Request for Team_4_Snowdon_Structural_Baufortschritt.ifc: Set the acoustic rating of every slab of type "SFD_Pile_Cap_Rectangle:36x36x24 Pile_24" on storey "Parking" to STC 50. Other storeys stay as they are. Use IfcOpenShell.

First a look at what the model holds.

```python
import ifcopenshell
import ifcopenshell.util.element

model = ifcopenshell.open("Team_4_Snowdon_Structural_Baufortschritt.ifc")
print(model.schema)
storey = next(s for s in model.by_type("IfcBuildingStorey") if s.Name == "Parking")
slabs = [e for e in ifcopenshell.util.element.get_decomposition(storey) if e.is_a("IfcSlab")]
seen = {}
for e in slabs:
    element_type = ifcopenshell.util.element.get_type(e)
    key = (element_type.Name if element_type != e and element_type else None, ifcopenshell.util.element.get_pset(e, "Pset_SlabCommon", "AcousticRating"))
    seen[key] = seen.get(key, 0) + 1
for (name, value), count in sorted(seen.items(), key=str):
    print(count, "x", name, "|", value)
```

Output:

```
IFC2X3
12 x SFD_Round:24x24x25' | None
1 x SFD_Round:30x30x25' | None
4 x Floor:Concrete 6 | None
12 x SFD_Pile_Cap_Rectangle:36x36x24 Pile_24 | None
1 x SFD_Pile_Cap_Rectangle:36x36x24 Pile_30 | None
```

```python
import ifcopenshell
import ifcopenshell.api.pset
import ifcopenshell.util.element

model = ifcopenshell.open("Team_4_Snowdon_Structural_Baufortschritt.ifc")

storey = next(s for s in model.by_type("IfcBuildingStorey") if s.Name == "Parking")
slabs = [e for e in ifcopenshell.util.element.get_decomposition(storey) if e.is_a("IfcSlab")]

count = 0
for e in slabs:
    element_type = ifcopenshell.util.element.get_type(e)
    if element_type in (None, e) or element_type.Name != "SFD_Pile_Cap_Rectangle:36x36x24 Pile_24":
        continue
    # add_pset returns the element's existing set when there is one.
    pset = ifcopenshell.api.pset.add_pset(model, product=e, name="Pset_SlabCommon")
    ifcopenshell.api.pset.edit_pset(model, pset=pset, properties={"AcousticRating": "STC 50"})
    count += 1

print(count, "slabs updated")

model.write("Team_4_Snowdon_Structural_Baufortschritt_edited.ifc")
```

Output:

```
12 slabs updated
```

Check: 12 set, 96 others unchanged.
